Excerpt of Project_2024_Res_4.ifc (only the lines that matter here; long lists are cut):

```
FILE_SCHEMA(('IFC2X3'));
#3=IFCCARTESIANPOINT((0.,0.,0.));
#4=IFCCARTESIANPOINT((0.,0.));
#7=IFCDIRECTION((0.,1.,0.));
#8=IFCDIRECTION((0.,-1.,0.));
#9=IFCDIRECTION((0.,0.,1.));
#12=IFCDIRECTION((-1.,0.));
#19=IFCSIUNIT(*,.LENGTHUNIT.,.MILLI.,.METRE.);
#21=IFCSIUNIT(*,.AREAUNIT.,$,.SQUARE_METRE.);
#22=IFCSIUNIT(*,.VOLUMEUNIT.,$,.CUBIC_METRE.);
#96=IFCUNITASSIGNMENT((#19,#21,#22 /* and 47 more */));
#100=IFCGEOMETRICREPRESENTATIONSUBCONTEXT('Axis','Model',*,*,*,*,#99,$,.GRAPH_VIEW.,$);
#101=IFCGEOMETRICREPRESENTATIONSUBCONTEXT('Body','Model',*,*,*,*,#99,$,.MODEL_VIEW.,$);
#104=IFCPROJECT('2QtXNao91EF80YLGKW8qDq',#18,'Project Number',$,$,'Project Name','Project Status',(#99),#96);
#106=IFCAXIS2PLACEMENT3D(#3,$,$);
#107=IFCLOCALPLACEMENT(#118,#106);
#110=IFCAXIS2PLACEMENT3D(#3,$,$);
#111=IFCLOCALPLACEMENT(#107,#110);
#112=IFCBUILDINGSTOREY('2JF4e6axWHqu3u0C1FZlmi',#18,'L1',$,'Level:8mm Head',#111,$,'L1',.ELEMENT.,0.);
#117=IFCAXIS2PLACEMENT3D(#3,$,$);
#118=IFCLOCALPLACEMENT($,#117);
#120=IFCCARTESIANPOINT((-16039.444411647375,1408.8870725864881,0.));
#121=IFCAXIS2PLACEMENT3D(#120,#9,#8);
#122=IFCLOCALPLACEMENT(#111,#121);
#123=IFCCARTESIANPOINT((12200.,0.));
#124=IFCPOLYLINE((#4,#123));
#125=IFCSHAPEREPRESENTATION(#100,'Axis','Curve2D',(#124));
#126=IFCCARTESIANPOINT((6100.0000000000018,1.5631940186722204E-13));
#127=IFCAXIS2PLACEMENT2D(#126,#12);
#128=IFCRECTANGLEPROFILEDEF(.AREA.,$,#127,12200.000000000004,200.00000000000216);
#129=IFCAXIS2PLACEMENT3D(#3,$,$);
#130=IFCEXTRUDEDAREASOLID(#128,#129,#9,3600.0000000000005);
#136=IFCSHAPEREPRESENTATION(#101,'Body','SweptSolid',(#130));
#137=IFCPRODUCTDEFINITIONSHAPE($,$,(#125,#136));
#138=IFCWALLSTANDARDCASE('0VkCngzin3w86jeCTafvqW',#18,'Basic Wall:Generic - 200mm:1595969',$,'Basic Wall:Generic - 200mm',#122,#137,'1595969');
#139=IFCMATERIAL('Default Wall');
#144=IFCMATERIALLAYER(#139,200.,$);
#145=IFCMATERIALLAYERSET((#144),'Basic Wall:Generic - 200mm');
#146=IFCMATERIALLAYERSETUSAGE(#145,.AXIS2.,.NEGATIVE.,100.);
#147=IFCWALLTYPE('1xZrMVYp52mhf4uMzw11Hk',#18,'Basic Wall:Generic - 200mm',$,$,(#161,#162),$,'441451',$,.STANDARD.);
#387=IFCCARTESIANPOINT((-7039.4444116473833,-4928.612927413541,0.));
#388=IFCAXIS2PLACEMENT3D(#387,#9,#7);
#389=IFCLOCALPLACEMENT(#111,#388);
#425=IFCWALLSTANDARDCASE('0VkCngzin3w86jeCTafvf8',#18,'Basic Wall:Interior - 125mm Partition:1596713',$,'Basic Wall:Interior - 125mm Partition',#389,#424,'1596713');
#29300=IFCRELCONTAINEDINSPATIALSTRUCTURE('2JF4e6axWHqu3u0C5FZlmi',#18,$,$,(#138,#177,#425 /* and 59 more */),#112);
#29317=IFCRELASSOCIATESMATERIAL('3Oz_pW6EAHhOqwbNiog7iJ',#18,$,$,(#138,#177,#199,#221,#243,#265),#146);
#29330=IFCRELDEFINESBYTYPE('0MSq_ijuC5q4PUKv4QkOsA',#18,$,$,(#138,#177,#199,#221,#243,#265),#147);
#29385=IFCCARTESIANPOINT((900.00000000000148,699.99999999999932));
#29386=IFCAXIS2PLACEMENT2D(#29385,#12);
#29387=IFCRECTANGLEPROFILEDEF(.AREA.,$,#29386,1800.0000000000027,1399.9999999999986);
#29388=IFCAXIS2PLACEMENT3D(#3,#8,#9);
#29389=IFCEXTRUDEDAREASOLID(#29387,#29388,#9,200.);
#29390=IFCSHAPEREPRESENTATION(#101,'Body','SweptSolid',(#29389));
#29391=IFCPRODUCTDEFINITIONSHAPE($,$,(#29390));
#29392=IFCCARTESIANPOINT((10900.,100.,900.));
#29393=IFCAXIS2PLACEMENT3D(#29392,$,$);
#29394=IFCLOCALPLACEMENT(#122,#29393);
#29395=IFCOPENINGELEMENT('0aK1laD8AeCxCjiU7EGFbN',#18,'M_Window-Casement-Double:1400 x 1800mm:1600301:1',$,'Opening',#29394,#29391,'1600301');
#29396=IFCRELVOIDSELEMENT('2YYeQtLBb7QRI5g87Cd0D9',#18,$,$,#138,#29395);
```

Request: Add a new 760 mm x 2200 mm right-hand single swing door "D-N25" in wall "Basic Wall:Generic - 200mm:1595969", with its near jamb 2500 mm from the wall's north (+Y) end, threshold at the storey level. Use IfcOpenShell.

```python
import numpy as np
import ifcopenshell
import ifcopenshell.api.feature
import ifcopenshell.api.geometry
import ifcopenshell.api.root
import ifcopenshell.api.spatial
import ifcopenshell.api.type
import ifcopenshell.geom
import ifcopenshell.util.element
import ifcopenshell.util.placement
import ifcopenshell.util.representation
import ifcopenshell.util.shape
import ifcopenshell.util.unit

model = ifcopenshell.open("Project_2024_Res_4.ifc")
unit_scale = ifcopenshell.util.unit.calculate_unit_scale(model)
settings = ifcopenshell.geom.settings()


def volume(element):
    """Net volume in cubic metres, openings subtracted."""
    shape = ifcopenshell.geom.create_shape(settings, element)
    return ifcopenshell.util.shape.get_volume(shape.geometry)


wall = model.by_guid("0VkCngzin3w86jeCTafvqW")
storey = ifcopenshell.util.element.get_container(wall, ifc_class="IfcBuildingStorey")
context = ifcopenshell.util.representation.get_context(model, "Model", "Body", "MODEL_VIEW")
before = volume(wall)

width, height, from_end, sill = 0.76, 2.2, 2.5, 0.0  # metres

# The wall runs along its own X axis, and the end named is its -X end.
wall_shape = ifcopenshell.geom.create_shape(settings, wall)
x, y, z = ifcopenshell.util.shape.get_vertices(wall_shape.geometry).T
start = x.min() + from_end
face, thickness = float(y.min()), float(y.max() - y.min())
wall_matrix = ifcopenshell.util.placement.get_local_placement(wall.ObjectPlacement)
level = ifcopenshell.util.placement.get_local_placement(storey.ObjectPlacement)[2, 3]


def in_wall(x, y):
    """Placement at x, y metres in the wall's axes, at sill height."""
    matrix = wall_matrix.copy()
    matrix[:, 3] = wall_matrix @ np.array([x / unit_scale, y / unit_scale, 0.0, 1.0])
    matrix[2, 3] = level + sill / unit_scale
    return matrix


# Opening: a box that overshoots both wall faces by 50 mm.
opening = ifcopenshell.api.root.create_entity(model, ifc_class="IfcOpeningElement")
box = ifcopenshell.api.geometry.add_wall_representation(
    model, context=context, length=width, height=height, thickness=thickness + 0.1
)
ifcopenshell.api.geometry.assign_representation(model, product=opening, representation=box)
ifcopenshell.api.geometry.edit_object_placement(model, product=opening, matrix=in_wall(start, face - 0.05), is_si=False)
ifcopenshell.api.feature.add_feature(model, feature=opening, element=wall)

door = ifcopenshell.api.root.create_entity(model, ifc_class="IfcDoor", name="D-N25")
door.OverallWidth, door.OverallHeight = width / unit_scale, height / unit_scale
body = ifcopenshell.api.geometry.add_door_representation(
    model,
    context=context,
    overall_width=door.OverallWidth,
    overall_height=door.OverallHeight,
    operation_type="SINGLE_SWING_RIGHT",
    lining_properties={"LiningDepth": thickness / unit_scale, "ThresholdDepth": thickness / unit_scale},
)
ifcopenshell.api.geometry.assign_representation(model, product=door, representation=body)
ifcopenshell.api.spatial.assign_container(model, products=[door], relating_structure=storey)
fills = ifcopenshell.api.feature.add_filling(model, opening=opening, element=door)
fills.OwnerHistory = door.OwnerHistory  # required in IFC2X3

# IFC2X3 keeps the operation on the door style.
style = ifcopenshell.api.root.create_entity(model, ifc_class="IfcDoorStyle", name="D-N25")
style.OperationType, style.ConstructionType = "SINGLE_SWING_RIGHT", "NOTDEFINED"
style.ParameterTakesPrecedence = style.Sizeable = False
ifcopenshell.api.type.assign_type(model, related_objects=[door], relating_type=style)

# The lining spans the wall, so the door starts at the wall face.
ifcopenshell.api.geometry.edit_object_placement(model, product=door, matrix=in_wall(start, face), is_si=False)

after = volume(wall)

print(f"wall volume {before:.3f} -> {after:.3f} m3")

model.write("Project_2024_Res_4_rev.ifc")
```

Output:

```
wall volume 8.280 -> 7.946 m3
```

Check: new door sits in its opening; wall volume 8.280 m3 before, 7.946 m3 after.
